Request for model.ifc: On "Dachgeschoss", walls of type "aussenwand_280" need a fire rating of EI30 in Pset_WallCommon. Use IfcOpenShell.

First a look at what the model holds.

```python
import ifcopenshell
import ifcopenshell.util.element

model = ifcopenshell.open("model.ifc")
print(model.schema)
storey = next(s for s in model.by_type("IfcBuildingStorey") if s.Name == "Dachgeschoss")
walls = [e for e in ifcopenshell.util.element.get_decomposition(storey) if e.is_a("IfcWall")]
seen = {}
for e in walls:
    element_type = ifcopenshell.util.element.get_type(e)
    key = (element_type.Name if element_type != e and element_type else None, ifcopenshell.util.element.get_pset(e, "Pset_WallCommon", "FireRating"))
    seen[key] = seen.get(key, 0) + 1
for (name, value), count in sorted(seen.items(), key=str):
    print(count, "x", name, "|", value)
```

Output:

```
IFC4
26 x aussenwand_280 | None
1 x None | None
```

```python
import ifcopenshell
import ifcopenshell.api.pset
import ifcopenshell.util.element

model = ifcopenshell.open("model.ifc")

storey = next(s for s in model.by_type("IfcBuildingStorey") if s.Name == "Dachgeschoss")
walls = [e for e in ifcopenshell.util.element.get_decomposition(storey) if e.is_a("IfcWall")]

count = 0
for e in walls:
    element_type = ifcopenshell.util.element.get_type(e)
    if element_type in (None, e) or element_type.Name != "aussenwand_280":
        continue
    # add_pset returns the element's existing set when there is one.
    pset = ifcopenshell.api.pset.add_pset(model, product=e, name="Pset_WallCommon")
    ifcopenshell.api.pset.edit_pset(model, pset=pset, properties={"FireRating": "EI30"})
    count += 1

print(count, "walls updated")

model.write("model_rev.ifc")
```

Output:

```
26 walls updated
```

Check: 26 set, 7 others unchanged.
